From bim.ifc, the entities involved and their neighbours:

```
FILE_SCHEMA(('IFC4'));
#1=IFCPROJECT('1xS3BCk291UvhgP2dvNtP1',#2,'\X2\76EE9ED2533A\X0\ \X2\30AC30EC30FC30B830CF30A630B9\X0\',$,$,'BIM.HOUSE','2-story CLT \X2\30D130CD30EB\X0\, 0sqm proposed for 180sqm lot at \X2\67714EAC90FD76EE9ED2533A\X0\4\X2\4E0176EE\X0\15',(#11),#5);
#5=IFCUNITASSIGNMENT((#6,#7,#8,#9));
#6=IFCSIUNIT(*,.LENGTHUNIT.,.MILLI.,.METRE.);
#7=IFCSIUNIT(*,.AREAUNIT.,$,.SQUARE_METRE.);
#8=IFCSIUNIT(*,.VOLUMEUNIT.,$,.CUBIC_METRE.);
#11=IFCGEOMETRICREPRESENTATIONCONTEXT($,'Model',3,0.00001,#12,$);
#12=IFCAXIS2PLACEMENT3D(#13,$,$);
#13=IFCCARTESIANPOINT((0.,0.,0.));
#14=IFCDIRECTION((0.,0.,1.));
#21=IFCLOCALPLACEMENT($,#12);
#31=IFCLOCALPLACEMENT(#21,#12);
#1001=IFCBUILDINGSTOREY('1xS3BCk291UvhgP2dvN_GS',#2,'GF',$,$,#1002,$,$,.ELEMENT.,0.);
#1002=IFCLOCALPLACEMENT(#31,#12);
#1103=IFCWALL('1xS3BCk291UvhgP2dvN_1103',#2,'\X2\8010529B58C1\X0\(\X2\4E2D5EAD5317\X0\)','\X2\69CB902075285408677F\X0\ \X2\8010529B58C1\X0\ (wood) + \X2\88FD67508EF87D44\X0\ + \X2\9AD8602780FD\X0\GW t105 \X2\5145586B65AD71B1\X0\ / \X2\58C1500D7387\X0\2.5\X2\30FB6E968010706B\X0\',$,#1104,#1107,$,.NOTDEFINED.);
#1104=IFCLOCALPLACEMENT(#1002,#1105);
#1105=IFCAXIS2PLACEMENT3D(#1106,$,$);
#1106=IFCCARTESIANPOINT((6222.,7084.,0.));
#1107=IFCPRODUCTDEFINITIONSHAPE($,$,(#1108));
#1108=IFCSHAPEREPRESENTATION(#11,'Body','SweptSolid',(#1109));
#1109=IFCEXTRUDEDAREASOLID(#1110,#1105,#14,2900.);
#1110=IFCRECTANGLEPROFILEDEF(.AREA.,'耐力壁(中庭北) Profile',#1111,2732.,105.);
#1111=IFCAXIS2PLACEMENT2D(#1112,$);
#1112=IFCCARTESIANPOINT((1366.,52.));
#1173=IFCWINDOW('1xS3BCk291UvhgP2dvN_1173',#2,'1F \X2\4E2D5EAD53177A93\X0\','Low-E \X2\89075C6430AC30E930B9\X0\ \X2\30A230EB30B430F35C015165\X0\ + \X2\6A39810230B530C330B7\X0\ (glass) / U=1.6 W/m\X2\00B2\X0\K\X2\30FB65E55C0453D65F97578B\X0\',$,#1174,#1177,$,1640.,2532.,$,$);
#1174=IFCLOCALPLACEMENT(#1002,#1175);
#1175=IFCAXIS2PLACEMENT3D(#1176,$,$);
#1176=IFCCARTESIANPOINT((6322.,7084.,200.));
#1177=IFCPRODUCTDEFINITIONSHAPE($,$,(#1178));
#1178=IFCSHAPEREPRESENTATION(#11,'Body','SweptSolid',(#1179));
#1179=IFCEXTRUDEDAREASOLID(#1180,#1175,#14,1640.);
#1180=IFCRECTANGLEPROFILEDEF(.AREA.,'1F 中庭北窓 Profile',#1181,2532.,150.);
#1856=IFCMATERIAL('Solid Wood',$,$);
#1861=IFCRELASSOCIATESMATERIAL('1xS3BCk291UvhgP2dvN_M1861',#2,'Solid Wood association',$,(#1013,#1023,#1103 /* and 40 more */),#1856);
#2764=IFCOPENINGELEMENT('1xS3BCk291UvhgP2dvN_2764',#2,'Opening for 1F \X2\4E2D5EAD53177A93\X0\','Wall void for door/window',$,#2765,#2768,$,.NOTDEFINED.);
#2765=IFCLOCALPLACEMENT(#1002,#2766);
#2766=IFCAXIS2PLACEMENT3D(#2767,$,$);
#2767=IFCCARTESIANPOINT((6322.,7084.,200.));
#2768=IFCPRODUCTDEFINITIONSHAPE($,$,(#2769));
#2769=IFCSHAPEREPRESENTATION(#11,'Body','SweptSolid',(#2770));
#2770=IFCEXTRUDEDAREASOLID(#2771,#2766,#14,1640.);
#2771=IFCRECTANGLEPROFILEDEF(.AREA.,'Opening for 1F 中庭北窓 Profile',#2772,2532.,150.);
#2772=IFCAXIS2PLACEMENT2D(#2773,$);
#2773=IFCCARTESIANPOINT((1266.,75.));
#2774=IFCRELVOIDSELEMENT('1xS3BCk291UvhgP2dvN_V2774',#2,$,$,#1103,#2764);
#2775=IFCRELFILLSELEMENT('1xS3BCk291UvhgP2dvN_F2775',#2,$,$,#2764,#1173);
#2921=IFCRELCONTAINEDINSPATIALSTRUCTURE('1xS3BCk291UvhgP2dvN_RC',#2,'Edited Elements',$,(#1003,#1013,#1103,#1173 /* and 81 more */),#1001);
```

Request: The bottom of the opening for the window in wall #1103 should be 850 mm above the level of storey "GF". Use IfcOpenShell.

```python
import numpy as np
import ifcopenshell
import ifcopenshell.api.geometry
import ifcopenshell.geom
import ifcopenshell.util.element
import ifcopenshell.util.placement
import ifcopenshell.util.shape
import ifcopenshell.util.unit

model = ifcopenshell.open("bim.ifc")
unit_scale = ifcopenshell.util.unit.calculate_unit_scale(model)

window = model.by_id(1173)
opening = window.FillsVoids[0].RelatingOpeningElement
storey = ifcopenshell.util.element.get_container(window, ifc_class="IfcBuildingStorey")
level = ifcopenshell.util.placement.get_local_placement(storey.ObjectPlacement)[2, 3]

# The opening's origin need not be at the sill, so measure its lowest point.
shape = ifcopenshell.geom.create_shape(ifcopenshell.geom.settings(), opening)
bottom = ifcopenshell.util.shape.get_shape_bottom_elevation(shape, shape.geometry) / unit_scale
dz = level + 0.85 / unit_scale - bottom

shift = np.array([0.0, 0.0, dz])
# The window is not placed relative to its opening, so move both.
for product in (opening, window):
    matrix = ifcopenshell.util.placement.get_local_placement(product.ObjectPlacement)
    matrix[:3, 3] += shift
    ifcopenshell.api.geometry.edit_object_placement(model, product=product, matrix=matrix, is_si=False)

print(f"moved by {dz * unit_scale:+.3f} m")

model.write("bim_edited.ifc")
```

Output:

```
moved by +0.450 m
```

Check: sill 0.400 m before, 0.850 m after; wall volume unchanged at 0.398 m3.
